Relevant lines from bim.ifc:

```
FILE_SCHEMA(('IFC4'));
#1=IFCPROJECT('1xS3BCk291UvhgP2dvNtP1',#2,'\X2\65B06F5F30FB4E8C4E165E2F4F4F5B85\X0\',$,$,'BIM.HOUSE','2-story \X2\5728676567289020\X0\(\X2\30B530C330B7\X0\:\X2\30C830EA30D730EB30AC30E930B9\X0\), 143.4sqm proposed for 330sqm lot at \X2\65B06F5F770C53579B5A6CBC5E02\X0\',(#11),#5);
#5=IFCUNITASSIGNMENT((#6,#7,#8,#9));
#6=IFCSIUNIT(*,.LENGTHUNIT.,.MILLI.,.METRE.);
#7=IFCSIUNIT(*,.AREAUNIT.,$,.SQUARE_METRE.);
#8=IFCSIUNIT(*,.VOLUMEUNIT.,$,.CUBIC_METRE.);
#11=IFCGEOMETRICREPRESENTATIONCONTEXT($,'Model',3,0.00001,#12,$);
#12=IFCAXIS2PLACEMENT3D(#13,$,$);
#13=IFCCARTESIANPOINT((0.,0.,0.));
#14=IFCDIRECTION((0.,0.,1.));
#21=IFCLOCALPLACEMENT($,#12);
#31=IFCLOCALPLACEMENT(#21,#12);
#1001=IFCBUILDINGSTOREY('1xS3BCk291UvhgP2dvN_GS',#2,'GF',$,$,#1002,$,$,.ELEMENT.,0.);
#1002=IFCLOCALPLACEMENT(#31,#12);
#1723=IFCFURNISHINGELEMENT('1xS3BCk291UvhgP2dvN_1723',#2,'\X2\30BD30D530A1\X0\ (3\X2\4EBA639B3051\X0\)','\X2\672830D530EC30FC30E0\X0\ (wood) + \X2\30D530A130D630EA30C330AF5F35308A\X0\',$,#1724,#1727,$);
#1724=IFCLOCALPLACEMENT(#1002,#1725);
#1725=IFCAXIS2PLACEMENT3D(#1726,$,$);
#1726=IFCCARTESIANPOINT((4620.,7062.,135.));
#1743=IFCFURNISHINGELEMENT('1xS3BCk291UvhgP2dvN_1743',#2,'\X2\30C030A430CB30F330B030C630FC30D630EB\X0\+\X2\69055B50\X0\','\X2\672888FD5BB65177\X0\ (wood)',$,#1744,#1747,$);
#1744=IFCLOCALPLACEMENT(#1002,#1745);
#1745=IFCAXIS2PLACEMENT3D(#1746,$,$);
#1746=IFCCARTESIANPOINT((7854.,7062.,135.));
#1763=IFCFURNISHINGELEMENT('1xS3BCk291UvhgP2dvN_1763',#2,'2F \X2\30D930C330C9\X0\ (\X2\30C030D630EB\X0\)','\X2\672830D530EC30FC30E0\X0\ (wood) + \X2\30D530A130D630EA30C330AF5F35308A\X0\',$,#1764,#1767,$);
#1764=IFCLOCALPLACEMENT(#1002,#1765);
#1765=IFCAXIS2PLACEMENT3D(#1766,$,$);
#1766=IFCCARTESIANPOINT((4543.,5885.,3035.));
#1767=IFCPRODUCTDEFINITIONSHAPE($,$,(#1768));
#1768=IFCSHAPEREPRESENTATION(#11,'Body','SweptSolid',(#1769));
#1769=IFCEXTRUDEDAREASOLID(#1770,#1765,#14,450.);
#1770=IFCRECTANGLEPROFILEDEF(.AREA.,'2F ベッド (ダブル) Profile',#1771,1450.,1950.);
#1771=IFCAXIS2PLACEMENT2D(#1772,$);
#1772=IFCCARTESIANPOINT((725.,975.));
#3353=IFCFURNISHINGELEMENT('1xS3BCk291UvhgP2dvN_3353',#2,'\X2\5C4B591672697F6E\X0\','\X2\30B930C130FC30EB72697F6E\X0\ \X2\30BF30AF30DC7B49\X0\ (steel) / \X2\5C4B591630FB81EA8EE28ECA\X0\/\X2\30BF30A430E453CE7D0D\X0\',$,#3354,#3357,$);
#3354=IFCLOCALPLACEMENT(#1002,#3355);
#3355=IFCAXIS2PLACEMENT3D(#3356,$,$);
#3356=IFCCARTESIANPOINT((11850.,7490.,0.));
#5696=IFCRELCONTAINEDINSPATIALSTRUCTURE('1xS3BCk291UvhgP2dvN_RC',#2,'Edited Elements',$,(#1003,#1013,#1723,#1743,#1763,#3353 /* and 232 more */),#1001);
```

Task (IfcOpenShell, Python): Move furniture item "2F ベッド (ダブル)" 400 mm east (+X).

```python
import ifcopenshell
import ifcopenshell.api.geometry
import ifcopenshell.util.placement

model = ifcopenshell.open("bim.ifc")

item = model.by_guid("1xS3BCk291UvhgP2dvN_1763")
matrix = ifcopenshell.util.placement.get_local_placement(item.ObjectPlacement)
matrix[0, 3] += 400.0
ifcopenshell.api.geometry.edit_object_placement(model, product=item, matrix=matrix, is_si=False)

print(ifcopenshell.util.placement.get_local_placement(item.ObjectPlacement).round(3) + 0.0)

model.write("bim-out.ifc")
```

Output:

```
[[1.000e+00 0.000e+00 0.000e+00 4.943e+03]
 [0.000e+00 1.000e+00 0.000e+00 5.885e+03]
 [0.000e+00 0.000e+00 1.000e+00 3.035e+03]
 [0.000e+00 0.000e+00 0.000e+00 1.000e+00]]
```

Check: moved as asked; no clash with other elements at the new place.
